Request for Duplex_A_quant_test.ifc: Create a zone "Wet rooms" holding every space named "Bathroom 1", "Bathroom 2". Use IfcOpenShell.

First a look at what the model holds.

```python
import ifcopenshell

model = ifcopenshell.open("Duplex_A_quant_test.ifc")
print(model.schema)
seen = {}
for space in model.by_type("IfcSpace"):
    seen[space.LongName] = seen.get(space.LongName, 0) + 1
for name, count in sorted(seen.items(), key=str):
    print(count, "x", name)
print("zones:", [z.Name for z in model.by_type("IfcZone")][:20])
```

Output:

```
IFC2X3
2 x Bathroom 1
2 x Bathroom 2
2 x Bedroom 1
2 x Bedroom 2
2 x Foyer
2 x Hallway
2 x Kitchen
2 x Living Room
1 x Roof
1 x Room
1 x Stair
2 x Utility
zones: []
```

```python
import ifcopenshell
import ifcopenshell.api.group
import ifcopenshell.api.root

model = ifcopenshell.open("Duplex_A_quant_test.ifc")

names = {"Bathroom 1", "Bathroom 2"}
spaces = [s for s in model.by_type("IfcSpace") if s.LongName in names]

zone = ifcopenshell.api.root.create_entity(model, ifc_class="IfcZone", name="Wet rooms")
ifcopenshell.api.group.assign_group(model, products=spaces, group=zone)
print(len(spaces), "spaces in", zone.Name)

model.write("Duplex_A_quant_test_edited.ifc")
```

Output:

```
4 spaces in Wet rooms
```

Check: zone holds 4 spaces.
